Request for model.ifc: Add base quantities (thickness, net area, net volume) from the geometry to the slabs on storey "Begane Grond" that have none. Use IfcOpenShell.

First a look at what the model holds.

```python
import ifcopenshell
import ifcopenshell.util.element
import ifcopenshell.util.unit

model = ifcopenshell.open("model.ifc")
print(model.schema)
for unit_type in ("LENGTHUNIT", "AREAUNIT", "VOLUMEUNIT"):
    print(unit_type, ifcopenshell.util.unit.calculate_unit_scale(model, unit_type))
storey = next(s for s in model.by_type("IfcBuildingStorey") if s.Name == "Begane Grond")
slabs = [e for e in ifcopenshell.util.element.get_decomposition(storey) if e.is_a("IfcSlab")]
for e in sorted(slabs, key=lambda e: e.id()):
    print(e.id(), e.is_a(), e.Name, list(ifcopenshell.util.element.get_psets(e, qtos_only=True)), sep=" | ")
```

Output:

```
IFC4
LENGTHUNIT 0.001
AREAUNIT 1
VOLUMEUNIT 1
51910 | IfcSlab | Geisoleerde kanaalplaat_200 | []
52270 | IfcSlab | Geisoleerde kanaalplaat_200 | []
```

```python
import ifcopenshell
import ifcopenshell.api.pset
import ifcopenshell.geom
import ifcopenshell.util.element
import ifcopenshell.util.shape
import ifcopenshell.util.unit

model = ifcopenshell.open("model.ifc")
unit_scale = ifcopenshell.util.unit.calculate_unit_scale(model)
area_scale = ifcopenshell.util.unit.calculate_unit_scale(model, "AREAUNIT")
volume_scale = ifcopenshell.util.unit.calculate_unit_scale(model, "VOLUMEUNIT")
settings = ifcopenshell.geom.settings()

storey = next(s for s in model.by_type("IfcBuildingStorey") if s.Name == "Begane Grond")
slabs = [e for e in ifcopenshell.util.element.get_decomposition(storey) if e.is_a("IfcSlab")]

for e in sorted(slabs, key=lambda e: e.id()):
    if ifcopenshell.util.element.get_psets(e, qtos_only=True, should_inherit=False):
        continue
    # Geometry comes back in metres, in the element's own axes.
    shape = ifcopenshell.geom.create_shape(settings, e)
    values = {
        "Width": ifcopenshell.util.shape.get_z(shape.geometry) / unit_scale,
        "NetArea": ifcopenshell.util.shape.get_footprint_area(shape.geometry) / area_scale,
        "NetVolume": ifcopenshell.util.shape.get_volume(shape.geometry) / volume_scale,
    }
    qto = ifcopenshell.api.pset.add_qto(model, product=e, name="Qto_SlabBaseQuantities")
    ifcopenshell.api.pset.edit_qto(model, qto=qto, properties=values)
    print(e.id(), {k: round(v, 3) for k, v in values.items()})

model.write("model_updated.ifc")
```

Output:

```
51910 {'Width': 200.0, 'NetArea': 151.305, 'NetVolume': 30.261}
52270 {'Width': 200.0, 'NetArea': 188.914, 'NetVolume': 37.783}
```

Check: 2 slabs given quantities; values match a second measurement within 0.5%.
